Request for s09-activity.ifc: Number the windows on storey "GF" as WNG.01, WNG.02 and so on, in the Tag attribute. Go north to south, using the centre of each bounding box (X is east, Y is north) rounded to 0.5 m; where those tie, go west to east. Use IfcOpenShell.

First a look at what the model holds.

```python
import ifcopenshell
import ifcopenshell.util.element
import ifcopenshell.util.placement

model = ifcopenshell.open("s09-activity.ifc")
print(model.schema)
storey = next(s for s in model.by_type("IfcBuildingStorey") if s.Name == "GF")
windows = [e for e in ifcopenshell.util.element.get_decomposition(storey) if e.is_a("IfcWindow")]
for e in sorted(windows, key=lambda e: e.id()):
    origin = ifcopenshell.util.placement.get_local_placement(e.ObjectPlacement)[:3, 3]
    print(e.id(), e.Tag, e.Name, origin.round(2) + 0.0, sep=" | ")
```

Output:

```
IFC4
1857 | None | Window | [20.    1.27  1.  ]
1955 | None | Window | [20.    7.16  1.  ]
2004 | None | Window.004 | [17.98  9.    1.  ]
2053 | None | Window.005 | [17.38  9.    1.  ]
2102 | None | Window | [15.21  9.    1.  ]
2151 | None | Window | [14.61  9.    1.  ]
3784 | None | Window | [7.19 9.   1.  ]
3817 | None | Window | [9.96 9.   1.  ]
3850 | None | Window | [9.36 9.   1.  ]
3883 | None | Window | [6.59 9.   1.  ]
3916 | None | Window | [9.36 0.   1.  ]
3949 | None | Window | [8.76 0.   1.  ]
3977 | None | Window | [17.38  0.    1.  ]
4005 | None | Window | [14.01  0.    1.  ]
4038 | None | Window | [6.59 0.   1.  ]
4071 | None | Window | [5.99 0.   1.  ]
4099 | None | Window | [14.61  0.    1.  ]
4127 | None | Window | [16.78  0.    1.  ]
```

```python
import ifcopenshell
import ifcopenshell.geom
import ifcopenshell.util.element
import ifcopenshell.util.shape

model = ifcopenshell.open("s09-activity.ifc")
settings = ifcopenshell.geom.settings()
settings.set("use-world-coords", True)


def centre(element):
    shape = ifcopenshell.geom.create_shape(settings, element)
    return ifcopenshell.util.shape.get_bbox_centroid(shape.geometry)


storey = next(s for s in model.by_type("IfcBuildingStorey") if s.Name == "GF")
windows = [e for e in ifcopenshell.util.element.get_decomposition(storey) if e.is_a("IfcWindow")]

# Insertion points can sit at a corner or the storey origin, so sort by the geometry (in metres).
centres = {e: centre(e) for e in windows}
windows.sort(key=lambda e: (-round(centres[e][1] / 0.5), centres[e][0]))

for i, e in enumerate(windows, start=1):
    number = f"WNG.{i:02d}"
    e.Tag = number
    print(e.id(), number)

model.write("s09-activity-out.ifc")
```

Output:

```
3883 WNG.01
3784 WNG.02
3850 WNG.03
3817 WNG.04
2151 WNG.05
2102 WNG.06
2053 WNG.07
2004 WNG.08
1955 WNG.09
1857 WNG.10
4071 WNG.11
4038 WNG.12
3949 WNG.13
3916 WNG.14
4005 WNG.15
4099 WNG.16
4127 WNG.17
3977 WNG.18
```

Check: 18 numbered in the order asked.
